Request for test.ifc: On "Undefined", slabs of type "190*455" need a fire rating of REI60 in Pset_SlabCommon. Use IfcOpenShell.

First a look at what the model holds.

```python
import ifcopenshell
import ifcopenshell.util.element

model = ifcopenshell.open("test.ifc")
print(model.schema)
storey = next(s for s in model.by_type("IfcBuildingStorey") if s.Name == "Undefined")
slabs = [e for e in ifcopenshell.util.element.get_decomposition(storey) if e.is_a("IfcSlab")]
seen = {}
for e in slabs:
    element_type = ifcopenshell.util.element.get_type(e)
    key = (element_type.Name if element_type != e and element_type else None, ifcopenshell.util.element.get_pset(e, "Pset_SlabCommon", "FireRating"))
    seen[key] = seen.get(key, 0) + 1
for (name, value), count in sorted(seen.items(), key=str):
    print(count, "x", name, "|", value)
```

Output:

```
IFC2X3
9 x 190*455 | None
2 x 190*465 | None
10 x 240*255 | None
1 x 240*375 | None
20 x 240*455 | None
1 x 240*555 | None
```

```python
import ifcopenshell
import ifcopenshell.api.pset
import ifcopenshell.util.element

model = ifcopenshell.open("test.ifc")

storey = next(s for s in model.by_type("IfcBuildingStorey") if s.Name == "Undefined")
slabs = [e for e in ifcopenshell.util.element.get_decomposition(storey) if e.is_a("IfcSlab")]

count = 0
for e in slabs:
    element_type = ifcopenshell.util.element.get_type(e)
    if element_type in (None, e) or element_type.Name != "190*455":
        continue
    found = ifcopenshell.util.element.get_pset(e, "Pset_SlabCommon", should_inherit=False)
    if found:
        pset = model.by_id(found["id"])
        if len(ifcopenshell.util.element.get_elements_by_pset(pset)) > 1:
            pset = ifcopenshell.api.pset.unshare_pset(model, products=[e], pset=pset)[0]
    else:
        pset = ifcopenshell.api.pset.add_pset(model, product=e, name="Pset_SlabCommon")
    ifcopenshell.api.pset.edit_pset(model, pset=pset, properties={"FireRating": "REI60"})
    count += 1

print(count, "slabs updated")

model.write("test_v2.ifc")
```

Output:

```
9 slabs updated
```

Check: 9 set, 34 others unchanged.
